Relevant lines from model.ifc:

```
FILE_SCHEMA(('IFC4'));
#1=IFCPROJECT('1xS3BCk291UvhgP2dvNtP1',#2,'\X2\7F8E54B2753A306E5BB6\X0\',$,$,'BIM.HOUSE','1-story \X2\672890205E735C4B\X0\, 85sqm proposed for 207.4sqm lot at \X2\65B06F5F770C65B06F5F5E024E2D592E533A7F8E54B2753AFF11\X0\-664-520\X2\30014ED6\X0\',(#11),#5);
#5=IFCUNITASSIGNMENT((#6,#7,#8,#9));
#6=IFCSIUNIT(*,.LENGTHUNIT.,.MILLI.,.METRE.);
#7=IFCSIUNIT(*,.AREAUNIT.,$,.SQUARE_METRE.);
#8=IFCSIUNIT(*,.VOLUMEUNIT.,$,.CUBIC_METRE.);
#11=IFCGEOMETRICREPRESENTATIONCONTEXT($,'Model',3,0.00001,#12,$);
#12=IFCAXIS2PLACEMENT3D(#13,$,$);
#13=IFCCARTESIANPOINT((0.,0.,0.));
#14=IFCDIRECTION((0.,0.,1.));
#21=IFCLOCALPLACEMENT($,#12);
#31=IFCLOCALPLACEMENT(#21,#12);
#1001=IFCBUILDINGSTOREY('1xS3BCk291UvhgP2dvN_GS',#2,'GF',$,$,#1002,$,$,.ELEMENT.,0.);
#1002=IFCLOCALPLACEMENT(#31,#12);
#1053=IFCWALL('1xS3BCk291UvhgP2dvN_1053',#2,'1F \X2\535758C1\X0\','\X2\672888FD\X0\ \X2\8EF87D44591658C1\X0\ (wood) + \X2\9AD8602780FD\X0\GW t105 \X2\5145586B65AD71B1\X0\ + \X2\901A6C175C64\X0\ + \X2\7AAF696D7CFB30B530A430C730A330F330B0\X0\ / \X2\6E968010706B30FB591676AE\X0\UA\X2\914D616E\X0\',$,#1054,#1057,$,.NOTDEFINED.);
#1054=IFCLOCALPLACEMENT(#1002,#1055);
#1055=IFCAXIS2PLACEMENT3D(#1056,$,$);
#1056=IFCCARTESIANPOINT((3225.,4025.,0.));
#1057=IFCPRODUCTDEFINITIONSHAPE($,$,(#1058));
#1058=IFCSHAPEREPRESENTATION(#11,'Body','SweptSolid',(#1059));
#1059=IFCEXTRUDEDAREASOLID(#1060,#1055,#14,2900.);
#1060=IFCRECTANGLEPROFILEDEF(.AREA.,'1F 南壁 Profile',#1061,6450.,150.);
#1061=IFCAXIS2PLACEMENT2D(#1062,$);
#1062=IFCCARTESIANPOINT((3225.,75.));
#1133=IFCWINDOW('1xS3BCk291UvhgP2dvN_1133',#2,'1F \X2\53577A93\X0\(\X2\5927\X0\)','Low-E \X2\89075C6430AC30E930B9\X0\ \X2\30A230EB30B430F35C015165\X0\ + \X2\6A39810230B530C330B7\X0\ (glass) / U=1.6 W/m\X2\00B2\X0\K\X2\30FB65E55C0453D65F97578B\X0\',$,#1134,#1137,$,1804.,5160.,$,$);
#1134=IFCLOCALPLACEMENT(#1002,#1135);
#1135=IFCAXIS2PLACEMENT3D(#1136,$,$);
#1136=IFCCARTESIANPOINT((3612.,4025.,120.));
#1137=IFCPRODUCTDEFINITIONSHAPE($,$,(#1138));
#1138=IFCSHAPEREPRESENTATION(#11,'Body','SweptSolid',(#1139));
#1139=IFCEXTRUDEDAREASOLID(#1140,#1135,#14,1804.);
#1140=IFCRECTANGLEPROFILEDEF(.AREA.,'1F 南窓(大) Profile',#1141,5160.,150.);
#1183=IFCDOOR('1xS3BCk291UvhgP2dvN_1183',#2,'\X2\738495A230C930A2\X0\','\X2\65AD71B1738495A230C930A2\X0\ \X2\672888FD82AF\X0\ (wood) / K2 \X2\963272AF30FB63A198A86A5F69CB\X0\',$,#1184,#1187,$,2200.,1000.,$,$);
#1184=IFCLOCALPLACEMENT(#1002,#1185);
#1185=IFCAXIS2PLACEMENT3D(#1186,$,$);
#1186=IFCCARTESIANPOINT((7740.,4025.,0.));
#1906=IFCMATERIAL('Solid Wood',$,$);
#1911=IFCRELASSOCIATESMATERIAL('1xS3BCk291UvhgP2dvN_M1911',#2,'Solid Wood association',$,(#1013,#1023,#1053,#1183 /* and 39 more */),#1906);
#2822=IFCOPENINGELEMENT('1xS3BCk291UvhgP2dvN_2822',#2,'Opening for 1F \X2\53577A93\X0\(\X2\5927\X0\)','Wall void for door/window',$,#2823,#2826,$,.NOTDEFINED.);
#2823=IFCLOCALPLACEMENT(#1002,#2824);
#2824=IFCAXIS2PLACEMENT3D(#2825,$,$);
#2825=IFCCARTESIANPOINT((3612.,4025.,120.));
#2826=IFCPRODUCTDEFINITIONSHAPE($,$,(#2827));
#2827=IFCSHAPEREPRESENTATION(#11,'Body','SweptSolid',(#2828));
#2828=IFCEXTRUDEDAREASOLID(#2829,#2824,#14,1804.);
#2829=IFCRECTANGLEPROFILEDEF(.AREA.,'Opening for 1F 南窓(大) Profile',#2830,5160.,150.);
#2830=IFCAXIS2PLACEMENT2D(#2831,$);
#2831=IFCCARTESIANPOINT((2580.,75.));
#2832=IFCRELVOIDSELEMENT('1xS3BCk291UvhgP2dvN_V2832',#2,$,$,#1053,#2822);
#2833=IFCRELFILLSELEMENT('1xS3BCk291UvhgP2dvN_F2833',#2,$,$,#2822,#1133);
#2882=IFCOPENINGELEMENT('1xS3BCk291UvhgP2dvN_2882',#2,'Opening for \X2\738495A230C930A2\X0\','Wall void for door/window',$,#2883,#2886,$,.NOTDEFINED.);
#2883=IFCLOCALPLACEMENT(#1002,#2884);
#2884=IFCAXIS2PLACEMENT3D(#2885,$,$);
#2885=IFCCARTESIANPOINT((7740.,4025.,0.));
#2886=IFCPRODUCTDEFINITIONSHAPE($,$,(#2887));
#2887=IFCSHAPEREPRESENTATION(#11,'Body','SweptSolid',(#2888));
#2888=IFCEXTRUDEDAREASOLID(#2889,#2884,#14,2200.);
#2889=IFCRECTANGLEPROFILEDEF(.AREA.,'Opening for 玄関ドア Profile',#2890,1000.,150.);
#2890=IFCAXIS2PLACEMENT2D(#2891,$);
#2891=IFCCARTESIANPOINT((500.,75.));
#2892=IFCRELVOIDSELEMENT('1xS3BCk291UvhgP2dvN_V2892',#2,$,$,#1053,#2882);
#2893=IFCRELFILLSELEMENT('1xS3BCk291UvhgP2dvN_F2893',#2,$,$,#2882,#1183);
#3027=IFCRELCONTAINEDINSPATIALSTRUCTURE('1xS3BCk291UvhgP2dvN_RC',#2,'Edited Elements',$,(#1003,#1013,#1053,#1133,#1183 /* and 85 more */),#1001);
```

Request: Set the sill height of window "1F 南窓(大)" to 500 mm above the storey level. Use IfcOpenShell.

```python
import numpy as np
import ifcopenshell
import ifcopenshell.api.geometry
import ifcopenshell.geom
import ifcopenshell.util.element
import ifcopenshell.util.placement
import ifcopenshell.util.shape
import ifcopenshell.util.unit

model = ifcopenshell.open("model.ifc")
unit_scale = ifcopenshell.util.unit.calculate_unit_scale(model)

window = model.by_guid("1xS3BCk291UvhgP2dvN_1133")
opening = window.FillsVoids[0].RelatingOpeningElement
storey = ifcopenshell.util.element.get_container(window, ifc_class="IfcBuildingStorey")
level = ifcopenshell.util.placement.get_local_placement(storey.ObjectPlacement)[2, 3]

# The opening's origin need not be at the sill, so measure its lowest point.
shape = ifcopenshell.geom.create_shape(ifcopenshell.geom.settings(), opening)
bottom = ifcopenshell.util.shape.get_shape_bottom_elevation(shape, shape.geometry) / unit_scale
dz = level + 500.0 - bottom

shift = np.array([0.0, 0.0, dz])
# The window is not placed relative to its opening, so move both.
for product in (opening, window):
    matrix = ifcopenshell.util.placement.get_local_placement(product.ObjectPlacement)
    matrix[:3, 3] += shift
    ifcopenshell.api.geometry.edit_object_placement(model, product=product, matrix=matrix, is_si=False)

print(f"moved by {dz * unit_scale:+.3f} m")

model.write("model-out.ifc")
```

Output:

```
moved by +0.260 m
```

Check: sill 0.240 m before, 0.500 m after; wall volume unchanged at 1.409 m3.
